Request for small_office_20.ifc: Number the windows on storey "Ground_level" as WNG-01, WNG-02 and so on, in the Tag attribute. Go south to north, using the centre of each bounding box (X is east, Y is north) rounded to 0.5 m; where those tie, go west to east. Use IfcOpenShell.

First a look at what the model holds.

```python
import ifcopenshell
import ifcopenshell.util.element
import ifcopenshell.util.placement

model = ifcopenshell.open("small_office_20.ifc")
print(model.schema)
storey = next(s for s in model.by_type("IfcBuildingStorey") if s.Name == "Ground_level")
windows = [e for e in ifcopenshell.util.element.get_decomposition(storey) if e.is_a("IfcWindow")]
for e in sorted(windows, key=lambda e: e.id()):
    origin = ifcopenshell.util.placement.get_local_placement(e.ObjectPlacement)[:3, 3]
    print(e.id(), e.Tag, e.Name, origin.round(2) + 0.0, sep=" | ")
```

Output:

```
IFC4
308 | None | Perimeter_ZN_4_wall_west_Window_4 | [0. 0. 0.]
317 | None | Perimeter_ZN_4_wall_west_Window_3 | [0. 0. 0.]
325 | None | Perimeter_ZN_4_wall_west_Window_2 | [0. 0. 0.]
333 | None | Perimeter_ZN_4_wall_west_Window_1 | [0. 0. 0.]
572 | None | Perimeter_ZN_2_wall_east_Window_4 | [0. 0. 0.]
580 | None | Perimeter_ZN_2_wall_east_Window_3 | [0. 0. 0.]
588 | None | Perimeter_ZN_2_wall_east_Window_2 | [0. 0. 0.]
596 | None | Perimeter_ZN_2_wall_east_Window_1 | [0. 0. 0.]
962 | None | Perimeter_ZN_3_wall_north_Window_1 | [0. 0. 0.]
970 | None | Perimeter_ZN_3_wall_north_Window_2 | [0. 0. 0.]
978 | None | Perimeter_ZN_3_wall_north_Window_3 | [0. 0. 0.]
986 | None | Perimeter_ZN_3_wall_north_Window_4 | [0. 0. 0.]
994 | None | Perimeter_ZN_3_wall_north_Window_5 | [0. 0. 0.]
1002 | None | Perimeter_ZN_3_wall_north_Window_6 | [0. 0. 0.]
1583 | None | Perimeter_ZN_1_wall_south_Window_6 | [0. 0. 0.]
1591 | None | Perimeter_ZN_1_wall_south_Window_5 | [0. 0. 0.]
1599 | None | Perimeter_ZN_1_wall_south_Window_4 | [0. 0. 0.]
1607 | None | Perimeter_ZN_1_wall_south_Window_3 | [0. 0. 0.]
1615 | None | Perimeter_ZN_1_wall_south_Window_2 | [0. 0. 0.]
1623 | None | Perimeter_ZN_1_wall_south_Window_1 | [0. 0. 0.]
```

```python
import ifcopenshell
import ifcopenshell.geom
import ifcopenshell.util.element
import ifcopenshell.util.shape

model = ifcopenshell.open("small_office_20.ifc")
settings = ifcopenshell.geom.settings()
settings.set("use-world-coords", True)


def centre(element):
    shape = ifcopenshell.geom.create_shape(settings, element)
    return ifcopenshell.util.shape.get_bbox_centroid(shape.geometry)


storey = next(s for s in model.by_type("IfcBuildingStorey") if s.Name == "Ground_level")
windows = [e for e in ifcopenshell.util.element.get_decomposition(storey) if e.is_a("IfcWindow")]

# Insertion points can sit at a corner or the storey origin, so sort by the geometry (in metres).
centres = {e: centre(e) for e in windows}
windows.sort(key=lambda e: (round(centres[e][1] / 0.5), centres[e][0]))

for i, e in enumerate(windows, start=1):
    number = f"WNG-{i:02d}"
    e.Tag = number
    print(e.id(), number)

model.write("small_office_20_updated.ifc")
```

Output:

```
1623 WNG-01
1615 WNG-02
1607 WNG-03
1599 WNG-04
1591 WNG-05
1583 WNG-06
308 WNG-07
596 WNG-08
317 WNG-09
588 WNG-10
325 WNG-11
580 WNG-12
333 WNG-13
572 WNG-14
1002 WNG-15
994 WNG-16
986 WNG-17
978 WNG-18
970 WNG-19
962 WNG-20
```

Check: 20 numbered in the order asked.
